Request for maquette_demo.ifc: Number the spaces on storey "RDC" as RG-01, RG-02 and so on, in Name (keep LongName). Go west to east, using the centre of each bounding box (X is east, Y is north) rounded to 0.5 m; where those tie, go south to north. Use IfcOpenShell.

First a look at what the model holds.

```python
import ifcopenshell
import ifcopenshell.util.element
import ifcopenshell.util.placement

model = ifcopenshell.open("maquette_demo.ifc")
print(model.schema)
storey = next(s for s in model.by_type("IfcBuildingStorey") if s.Name == "RDC")
spaces = [e for e in ifcopenshell.util.element.get_decomposition(storey) if e.is_a("IfcSpace")]
for e in sorted(spaces, key=lambda e: e.id()):
    origin = ifcopenshell.util.placement.get_local_placement(e.ObjectPlacement)[:3, 3]
    print(e.id(), e.Name, e.LongName, origin.round(2) + 0.0, sep=" | ")
```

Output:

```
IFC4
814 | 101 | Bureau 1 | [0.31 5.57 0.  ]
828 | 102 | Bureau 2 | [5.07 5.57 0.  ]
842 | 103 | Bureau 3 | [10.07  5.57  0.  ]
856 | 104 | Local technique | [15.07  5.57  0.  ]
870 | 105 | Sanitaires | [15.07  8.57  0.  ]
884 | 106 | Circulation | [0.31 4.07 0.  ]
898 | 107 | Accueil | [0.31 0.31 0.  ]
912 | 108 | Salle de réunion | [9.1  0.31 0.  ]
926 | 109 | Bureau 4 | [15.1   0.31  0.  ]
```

```python
import ifcopenshell
import ifcopenshell.geom
import ifcopenshell.util.element
import ifcopenshell.util.shape

model = ifcopenshell.open("maquette_demo.ifc")
settings = ifcopenshell.geom.settings()
settings.set("use-world-coords", True)


def centre(element):
    shape = ifcopenshell.geom.create_shape(settings, element)
    return ifcopenshell.util.shape.get_bbox_centroid(shape.geometry)


storey = next(s for s in model.by_type("IfcBuildingStorey") if s.Name == "RDC")
spaces = [e for e in ifcopenshell.util.element.get_decomposition(storey) if e.is_a("IfcSpace")]

# Insertion points can sit at a corner or the storey origin, so sort by the geometry (in metres).
centres = {e: centre(e) for e in spaces}
spaces.sort(key=lambda e: (round(centres[e][0] / 0.5), centres[e][1]))

for i, e in enumerate(spaces, start=1):
    number = f"RG-{i:02d}"
    e.Name = number
    print(e.id(), number)

model.write("maquette_demo_updated.ifc")
```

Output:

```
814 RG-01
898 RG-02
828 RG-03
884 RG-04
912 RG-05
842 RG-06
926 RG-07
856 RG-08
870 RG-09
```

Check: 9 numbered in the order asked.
